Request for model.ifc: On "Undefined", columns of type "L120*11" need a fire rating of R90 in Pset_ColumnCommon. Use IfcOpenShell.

First a look at what the model holds.

```python
import ifcopenshell
import ifcopenshell.util.element

model = ifcopenshell.open("model.ifc")
print(model.schema)
storey = next(s for s in model.by_type("IfcBuildingStorey") if s.Name == "Undefined")
columns = [e for e in ifcopenshell.util.element.get_decomposition(storey) if e.is_a("IfcColumn")]
seen = {}
for e in columns:
    element_type = ifcopenshell.util.element.get_type(e)
    key = (element_type.Name if element_type != e and element_type else None, ifcopenshell.util.element.get_pset(e, "Pset_ColumnCommon", "FireRating"))
    seen[key] = seen.get(key, 0) + 1
for (name, value), count in sorted(seen.items(), key=str):
    print(count, "x", name, "|", value)
```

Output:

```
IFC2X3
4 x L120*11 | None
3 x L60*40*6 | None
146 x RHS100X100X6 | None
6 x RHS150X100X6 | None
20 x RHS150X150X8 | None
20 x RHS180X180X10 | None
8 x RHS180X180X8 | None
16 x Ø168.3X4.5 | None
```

```python
import ifcopenshell
import ifcopenshell.api.pset
import ifcopenshell.util.element

model = ifcopenshell.open("model.ifc")

storey = next(s for s in model.by_type("IfcBuildingStorey") if s.Name == "Undefined")
columns = [e for e in ifcopenshell.util.element.get_decomposition(storey) if e.is_a("IfcColumn")]

count = 0
for e in columns:
    element_type = ifcopenshell.util.element.get_type(e)
    if element_type in (None, e) or element_type.Name != "L120*11":
        continue
    found = ifcopenshell.util.element.get_pset(e, "Pset_ColumnCommon", should_inherit=False)
    if found:
        pset = model.by_id(found["id"])
        if len(ifcopenshell.util.element.get_elements_by_pset(pset)) > 1:
            pset = ifcopenshell.api.pset.unshare_pset(model, products=[e], pset=pset)[0]
    else:
        pset = ifcopenshell.api.pset.add_pset(model, product=e, name="Pset_ColumnCommon")
    ifcopenshell.api.pset.edit_pset(model, pset=pset, properties={"FireRating": "R90"})
    count += 1

print(count, "columns updated")

model.write("model_rev.ifc")
```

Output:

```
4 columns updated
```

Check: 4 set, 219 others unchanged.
